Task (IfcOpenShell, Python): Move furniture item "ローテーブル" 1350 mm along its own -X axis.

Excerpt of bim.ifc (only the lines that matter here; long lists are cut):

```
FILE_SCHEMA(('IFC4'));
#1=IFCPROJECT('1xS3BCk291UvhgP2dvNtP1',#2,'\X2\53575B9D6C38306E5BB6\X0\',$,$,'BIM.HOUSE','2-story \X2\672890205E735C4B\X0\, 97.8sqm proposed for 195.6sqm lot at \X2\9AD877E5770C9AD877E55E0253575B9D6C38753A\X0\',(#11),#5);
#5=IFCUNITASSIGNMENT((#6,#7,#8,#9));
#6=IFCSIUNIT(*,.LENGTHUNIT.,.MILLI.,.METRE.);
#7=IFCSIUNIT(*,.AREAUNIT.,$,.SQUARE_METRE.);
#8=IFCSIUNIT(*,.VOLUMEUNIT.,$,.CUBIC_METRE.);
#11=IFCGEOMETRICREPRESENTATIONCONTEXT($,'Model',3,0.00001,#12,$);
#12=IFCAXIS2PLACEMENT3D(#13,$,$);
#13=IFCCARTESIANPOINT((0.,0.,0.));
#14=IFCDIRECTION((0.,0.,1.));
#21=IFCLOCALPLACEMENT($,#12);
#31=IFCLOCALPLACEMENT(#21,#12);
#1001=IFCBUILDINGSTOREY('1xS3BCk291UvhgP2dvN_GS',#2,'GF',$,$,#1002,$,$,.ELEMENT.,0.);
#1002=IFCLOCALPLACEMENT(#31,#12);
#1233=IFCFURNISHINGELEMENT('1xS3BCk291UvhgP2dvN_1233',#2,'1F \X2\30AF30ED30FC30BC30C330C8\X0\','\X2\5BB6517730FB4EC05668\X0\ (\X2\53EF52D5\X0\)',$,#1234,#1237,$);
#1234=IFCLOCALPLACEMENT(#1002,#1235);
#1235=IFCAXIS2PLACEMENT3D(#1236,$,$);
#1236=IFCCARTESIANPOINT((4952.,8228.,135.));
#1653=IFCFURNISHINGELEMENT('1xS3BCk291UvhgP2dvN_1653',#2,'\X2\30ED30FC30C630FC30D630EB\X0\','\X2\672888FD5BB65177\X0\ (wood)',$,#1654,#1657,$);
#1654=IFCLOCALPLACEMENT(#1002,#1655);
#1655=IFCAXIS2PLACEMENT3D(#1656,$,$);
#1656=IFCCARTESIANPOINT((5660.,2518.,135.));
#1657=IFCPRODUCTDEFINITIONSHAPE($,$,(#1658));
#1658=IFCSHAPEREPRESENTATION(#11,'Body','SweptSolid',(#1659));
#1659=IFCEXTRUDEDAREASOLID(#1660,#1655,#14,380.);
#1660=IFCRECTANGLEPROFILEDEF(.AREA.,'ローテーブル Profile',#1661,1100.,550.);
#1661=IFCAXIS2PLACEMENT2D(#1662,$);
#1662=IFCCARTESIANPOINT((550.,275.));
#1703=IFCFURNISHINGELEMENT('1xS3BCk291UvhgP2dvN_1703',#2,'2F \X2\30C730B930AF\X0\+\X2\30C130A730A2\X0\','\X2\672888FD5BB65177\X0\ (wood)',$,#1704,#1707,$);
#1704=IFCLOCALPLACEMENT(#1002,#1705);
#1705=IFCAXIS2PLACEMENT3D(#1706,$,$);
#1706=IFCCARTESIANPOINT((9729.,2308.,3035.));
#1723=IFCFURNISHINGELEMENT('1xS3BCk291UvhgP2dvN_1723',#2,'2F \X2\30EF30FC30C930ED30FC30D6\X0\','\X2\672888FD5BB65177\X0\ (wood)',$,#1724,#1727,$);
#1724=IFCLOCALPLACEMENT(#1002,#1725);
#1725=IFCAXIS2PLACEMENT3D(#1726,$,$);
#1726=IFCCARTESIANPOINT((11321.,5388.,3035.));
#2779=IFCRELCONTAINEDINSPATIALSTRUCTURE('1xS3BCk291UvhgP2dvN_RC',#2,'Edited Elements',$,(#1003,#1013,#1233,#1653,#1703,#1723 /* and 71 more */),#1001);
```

```python
import ifcopenshell
import ifcopenshell.api.geometry
import ifcopenshell.util.placement

model = ifcopenshell.open("bim.ifc")

item = model.by_id(1653)
matrix = ifcopenshell.util.placement.get_local_placement(item.ObjectPlacement)
matrix[:3, 3] -= matrix[:3, 0] * 1350.0
ifcopenshell.api.geometry.edit_object_placement(model, product=item, matrix=matrix, is_si=False)

print(ifcopenshell.util.placement.get_local_placement(item.ObjectPlacement).round(3) + 0.0)

model.write("bim-out.ifc")
```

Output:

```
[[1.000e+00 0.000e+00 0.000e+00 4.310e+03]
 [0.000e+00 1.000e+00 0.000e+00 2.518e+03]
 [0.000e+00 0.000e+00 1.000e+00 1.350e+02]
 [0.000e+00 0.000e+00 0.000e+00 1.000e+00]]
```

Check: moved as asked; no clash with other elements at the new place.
